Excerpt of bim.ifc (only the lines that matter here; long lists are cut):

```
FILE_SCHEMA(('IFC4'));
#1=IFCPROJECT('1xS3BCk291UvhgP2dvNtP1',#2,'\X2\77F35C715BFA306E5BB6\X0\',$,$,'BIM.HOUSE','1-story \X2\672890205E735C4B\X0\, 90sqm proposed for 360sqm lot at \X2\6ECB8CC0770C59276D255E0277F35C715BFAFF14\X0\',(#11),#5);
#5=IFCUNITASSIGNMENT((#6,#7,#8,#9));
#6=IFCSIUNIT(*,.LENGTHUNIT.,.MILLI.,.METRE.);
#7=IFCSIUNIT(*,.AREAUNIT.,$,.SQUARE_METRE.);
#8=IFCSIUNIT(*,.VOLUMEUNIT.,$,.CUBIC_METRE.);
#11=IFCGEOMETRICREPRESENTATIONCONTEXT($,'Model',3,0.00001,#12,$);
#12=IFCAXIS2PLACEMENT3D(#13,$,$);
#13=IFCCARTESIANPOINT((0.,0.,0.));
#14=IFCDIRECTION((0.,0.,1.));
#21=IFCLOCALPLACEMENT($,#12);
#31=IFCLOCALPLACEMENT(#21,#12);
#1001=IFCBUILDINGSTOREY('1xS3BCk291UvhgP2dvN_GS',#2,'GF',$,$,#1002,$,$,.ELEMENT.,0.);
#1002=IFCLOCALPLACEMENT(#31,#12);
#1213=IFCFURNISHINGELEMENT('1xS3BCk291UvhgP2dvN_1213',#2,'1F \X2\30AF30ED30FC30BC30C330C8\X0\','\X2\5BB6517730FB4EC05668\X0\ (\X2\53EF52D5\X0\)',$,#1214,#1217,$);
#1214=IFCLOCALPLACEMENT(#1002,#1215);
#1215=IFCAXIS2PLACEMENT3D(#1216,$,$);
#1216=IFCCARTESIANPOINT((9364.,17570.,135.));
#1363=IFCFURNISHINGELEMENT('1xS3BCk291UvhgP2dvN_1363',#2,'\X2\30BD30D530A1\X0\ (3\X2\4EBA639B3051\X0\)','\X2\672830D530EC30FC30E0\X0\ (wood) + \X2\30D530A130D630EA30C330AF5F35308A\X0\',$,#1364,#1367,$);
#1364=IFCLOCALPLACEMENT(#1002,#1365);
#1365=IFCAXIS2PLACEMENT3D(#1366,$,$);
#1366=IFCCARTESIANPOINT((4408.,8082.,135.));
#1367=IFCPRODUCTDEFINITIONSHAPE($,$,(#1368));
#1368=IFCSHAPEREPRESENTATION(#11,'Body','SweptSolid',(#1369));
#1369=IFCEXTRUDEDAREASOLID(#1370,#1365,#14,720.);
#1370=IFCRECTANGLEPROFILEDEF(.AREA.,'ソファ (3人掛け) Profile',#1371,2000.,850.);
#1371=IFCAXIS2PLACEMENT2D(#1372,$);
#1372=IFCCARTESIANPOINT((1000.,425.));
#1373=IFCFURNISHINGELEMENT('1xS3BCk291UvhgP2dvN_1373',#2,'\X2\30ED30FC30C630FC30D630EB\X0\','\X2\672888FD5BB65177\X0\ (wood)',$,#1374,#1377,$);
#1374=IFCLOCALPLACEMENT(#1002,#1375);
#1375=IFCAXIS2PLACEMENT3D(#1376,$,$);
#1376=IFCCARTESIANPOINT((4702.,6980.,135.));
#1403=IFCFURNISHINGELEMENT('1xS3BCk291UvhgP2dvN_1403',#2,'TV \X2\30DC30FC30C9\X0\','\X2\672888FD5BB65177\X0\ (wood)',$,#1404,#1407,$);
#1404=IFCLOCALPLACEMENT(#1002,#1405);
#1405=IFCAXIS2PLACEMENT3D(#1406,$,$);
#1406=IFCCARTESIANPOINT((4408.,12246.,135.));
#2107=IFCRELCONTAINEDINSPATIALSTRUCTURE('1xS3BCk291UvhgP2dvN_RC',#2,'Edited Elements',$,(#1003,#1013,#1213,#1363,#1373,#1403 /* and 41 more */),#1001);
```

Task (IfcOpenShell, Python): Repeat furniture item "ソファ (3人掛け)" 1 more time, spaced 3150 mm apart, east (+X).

```python
import numpy as np
import ifcopenshell
import ifcopenshell.api.geometry
import ifcopenshell.api.root
import ifcopenshell.util.element
import ifcopenshell.util.placement

model = ifcopenshell.open("bim.ifc")


def reuse_history(source, copy):
    """copy_class also copies each property set's owner history, people and application; keep the originals."""
    for rel in copy.IsDefinedBy:
        if rel.is_a("IfcRelDefinesByProperties") and (history := rel.RelatingPropertyDefinition.OwnerHistory):
            rel.RelatingPropertyDefinition.OwnerHistory = source.OwnerHistory
            ifcopenshell.util.element.remove_deep2(model, history)


source = model.by_guid("1xS3BCk291UvhgP2dvN_1363")
base = ifcopenshell.util.placement.get_local_placement(source.ObjectPlacement)
step = np.array([1.0, 0.0, 0.0]) * 3150.0

for i in range(1, 2):
    copy = ifcopenshell.api.root.copy_class(model, product=source)
    copy.Representation = ifcopenshell.util.element.copy_deep(
        model, source.Representation, exclude=["IfcGeometricRepresentationContext", "IfcRepresentationMap"]
    )
    reuse_history(source, copy)
    matrix = base.copy()
    matrix[:3, 3] += i * step
    print("added at", matrix[:3, 3].round(3) + 0.0)
    ifcopenshell.api.geometry.edit_object_placement(model, product=copy, matrix=matrix, is_si=False)

model.write("bim_v2.ifc")
```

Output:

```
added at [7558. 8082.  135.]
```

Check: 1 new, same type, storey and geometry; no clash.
